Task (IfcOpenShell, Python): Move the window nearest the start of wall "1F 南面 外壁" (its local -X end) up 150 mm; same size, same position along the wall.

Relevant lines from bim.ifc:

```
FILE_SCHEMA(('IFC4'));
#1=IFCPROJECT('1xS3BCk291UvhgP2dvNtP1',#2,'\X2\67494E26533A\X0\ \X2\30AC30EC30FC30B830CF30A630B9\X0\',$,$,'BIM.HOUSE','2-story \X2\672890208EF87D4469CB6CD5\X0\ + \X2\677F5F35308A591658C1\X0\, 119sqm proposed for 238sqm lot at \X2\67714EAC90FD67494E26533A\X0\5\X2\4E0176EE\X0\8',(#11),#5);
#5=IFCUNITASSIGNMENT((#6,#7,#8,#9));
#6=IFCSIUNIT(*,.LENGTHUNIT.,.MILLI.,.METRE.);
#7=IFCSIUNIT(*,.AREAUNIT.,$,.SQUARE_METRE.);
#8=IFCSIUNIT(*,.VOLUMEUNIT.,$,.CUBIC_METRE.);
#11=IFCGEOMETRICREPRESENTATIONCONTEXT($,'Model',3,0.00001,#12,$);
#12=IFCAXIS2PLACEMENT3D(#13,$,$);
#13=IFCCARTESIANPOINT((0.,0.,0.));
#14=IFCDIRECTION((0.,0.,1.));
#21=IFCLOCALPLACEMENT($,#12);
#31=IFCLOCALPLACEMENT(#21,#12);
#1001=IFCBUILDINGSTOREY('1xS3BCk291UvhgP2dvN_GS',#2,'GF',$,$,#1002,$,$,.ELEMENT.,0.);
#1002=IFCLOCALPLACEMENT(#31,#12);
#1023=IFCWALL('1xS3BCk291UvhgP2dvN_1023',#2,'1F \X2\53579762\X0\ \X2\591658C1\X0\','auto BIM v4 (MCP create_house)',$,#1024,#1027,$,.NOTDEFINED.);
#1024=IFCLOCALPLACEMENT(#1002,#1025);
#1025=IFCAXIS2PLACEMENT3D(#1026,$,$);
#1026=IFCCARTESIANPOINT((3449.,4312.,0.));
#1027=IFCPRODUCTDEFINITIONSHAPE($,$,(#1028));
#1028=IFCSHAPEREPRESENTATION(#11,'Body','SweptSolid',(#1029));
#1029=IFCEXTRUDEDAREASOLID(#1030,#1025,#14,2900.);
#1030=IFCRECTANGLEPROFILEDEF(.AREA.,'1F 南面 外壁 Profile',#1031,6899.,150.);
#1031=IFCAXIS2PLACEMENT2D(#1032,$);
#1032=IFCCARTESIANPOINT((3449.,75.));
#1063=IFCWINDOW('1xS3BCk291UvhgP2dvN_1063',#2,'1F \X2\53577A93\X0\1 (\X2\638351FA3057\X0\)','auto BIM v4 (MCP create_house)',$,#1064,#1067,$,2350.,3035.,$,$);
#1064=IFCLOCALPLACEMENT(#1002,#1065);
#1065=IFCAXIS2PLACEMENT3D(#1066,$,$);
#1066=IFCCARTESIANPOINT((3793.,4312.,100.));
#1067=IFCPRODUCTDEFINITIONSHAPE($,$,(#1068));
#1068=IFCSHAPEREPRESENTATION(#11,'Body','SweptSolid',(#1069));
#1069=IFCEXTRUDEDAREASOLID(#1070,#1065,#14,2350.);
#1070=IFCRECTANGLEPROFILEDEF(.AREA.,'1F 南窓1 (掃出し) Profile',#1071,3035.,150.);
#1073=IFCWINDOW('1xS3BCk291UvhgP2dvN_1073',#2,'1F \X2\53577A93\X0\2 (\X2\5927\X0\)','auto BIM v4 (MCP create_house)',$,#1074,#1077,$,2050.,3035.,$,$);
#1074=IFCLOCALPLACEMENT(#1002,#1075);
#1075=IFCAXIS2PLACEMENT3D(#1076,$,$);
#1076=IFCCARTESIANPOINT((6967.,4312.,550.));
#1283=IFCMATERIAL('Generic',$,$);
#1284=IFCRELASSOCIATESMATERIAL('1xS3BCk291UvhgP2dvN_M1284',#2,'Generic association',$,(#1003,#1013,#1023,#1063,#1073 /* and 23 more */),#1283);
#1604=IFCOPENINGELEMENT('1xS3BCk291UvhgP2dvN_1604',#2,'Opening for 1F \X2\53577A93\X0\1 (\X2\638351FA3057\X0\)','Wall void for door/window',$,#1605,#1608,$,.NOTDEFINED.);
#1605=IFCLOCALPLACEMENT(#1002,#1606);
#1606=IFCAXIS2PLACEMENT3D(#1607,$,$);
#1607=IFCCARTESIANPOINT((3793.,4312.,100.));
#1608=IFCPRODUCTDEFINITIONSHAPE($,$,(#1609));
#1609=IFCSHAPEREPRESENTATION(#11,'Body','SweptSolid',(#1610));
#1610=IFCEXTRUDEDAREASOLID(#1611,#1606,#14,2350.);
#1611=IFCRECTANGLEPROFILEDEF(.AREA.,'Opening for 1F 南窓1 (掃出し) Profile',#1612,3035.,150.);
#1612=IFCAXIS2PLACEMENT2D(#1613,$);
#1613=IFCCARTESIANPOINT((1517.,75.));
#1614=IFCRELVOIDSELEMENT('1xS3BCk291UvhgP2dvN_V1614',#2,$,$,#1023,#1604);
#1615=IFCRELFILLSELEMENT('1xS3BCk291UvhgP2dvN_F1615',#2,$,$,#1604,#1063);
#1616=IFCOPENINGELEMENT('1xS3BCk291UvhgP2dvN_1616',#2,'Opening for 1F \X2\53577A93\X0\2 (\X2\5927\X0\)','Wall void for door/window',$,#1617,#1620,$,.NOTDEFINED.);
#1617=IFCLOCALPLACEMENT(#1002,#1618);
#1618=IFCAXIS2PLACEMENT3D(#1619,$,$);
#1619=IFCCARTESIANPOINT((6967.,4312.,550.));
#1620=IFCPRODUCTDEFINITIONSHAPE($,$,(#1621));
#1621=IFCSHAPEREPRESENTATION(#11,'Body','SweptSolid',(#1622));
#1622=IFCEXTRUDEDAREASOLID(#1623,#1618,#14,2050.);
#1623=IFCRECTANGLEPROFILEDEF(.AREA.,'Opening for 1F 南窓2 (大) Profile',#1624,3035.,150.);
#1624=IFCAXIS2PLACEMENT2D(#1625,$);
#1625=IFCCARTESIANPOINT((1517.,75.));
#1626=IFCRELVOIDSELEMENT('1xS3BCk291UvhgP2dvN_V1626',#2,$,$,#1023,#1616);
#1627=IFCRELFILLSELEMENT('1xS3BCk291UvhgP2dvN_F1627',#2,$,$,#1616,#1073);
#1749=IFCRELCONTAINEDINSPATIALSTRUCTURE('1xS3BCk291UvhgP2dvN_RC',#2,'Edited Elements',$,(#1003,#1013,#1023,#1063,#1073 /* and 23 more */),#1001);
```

```python
import numpy as np
import ifcopenshell
import ifcopenshell.api.geometry
import ifcopenshell.util.placement
import ifcopenshell.util.unit

model = ifcopenshell.open("bim.ifc")
unit_scale = ifcopenshell.util.unit.calculate_unit_scale(model)

window = model.by_id(1063)
opening = window.FillsVoids[0].RelatingOpeningElement
dz = 0.15 / unit_scale

shift = np.array([0.0, 0.0, dz])
# The window is not placed relative to its opening, so move both.
for product in (opening, window):
    matrix = ifcopenshell.util.placement.get_local_placement(product.ObjectPlacement)
    matrix[:3, 3] += shift
    ifcopenshell.api.geometry.edit_object_placement(model, product=product, matrix=matrix, is_si=False)

print(f"moved by {dz * unit_scale:+.3f} m")

model.write("bim_v2.ifc")
```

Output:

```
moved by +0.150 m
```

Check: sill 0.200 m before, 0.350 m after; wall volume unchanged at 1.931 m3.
